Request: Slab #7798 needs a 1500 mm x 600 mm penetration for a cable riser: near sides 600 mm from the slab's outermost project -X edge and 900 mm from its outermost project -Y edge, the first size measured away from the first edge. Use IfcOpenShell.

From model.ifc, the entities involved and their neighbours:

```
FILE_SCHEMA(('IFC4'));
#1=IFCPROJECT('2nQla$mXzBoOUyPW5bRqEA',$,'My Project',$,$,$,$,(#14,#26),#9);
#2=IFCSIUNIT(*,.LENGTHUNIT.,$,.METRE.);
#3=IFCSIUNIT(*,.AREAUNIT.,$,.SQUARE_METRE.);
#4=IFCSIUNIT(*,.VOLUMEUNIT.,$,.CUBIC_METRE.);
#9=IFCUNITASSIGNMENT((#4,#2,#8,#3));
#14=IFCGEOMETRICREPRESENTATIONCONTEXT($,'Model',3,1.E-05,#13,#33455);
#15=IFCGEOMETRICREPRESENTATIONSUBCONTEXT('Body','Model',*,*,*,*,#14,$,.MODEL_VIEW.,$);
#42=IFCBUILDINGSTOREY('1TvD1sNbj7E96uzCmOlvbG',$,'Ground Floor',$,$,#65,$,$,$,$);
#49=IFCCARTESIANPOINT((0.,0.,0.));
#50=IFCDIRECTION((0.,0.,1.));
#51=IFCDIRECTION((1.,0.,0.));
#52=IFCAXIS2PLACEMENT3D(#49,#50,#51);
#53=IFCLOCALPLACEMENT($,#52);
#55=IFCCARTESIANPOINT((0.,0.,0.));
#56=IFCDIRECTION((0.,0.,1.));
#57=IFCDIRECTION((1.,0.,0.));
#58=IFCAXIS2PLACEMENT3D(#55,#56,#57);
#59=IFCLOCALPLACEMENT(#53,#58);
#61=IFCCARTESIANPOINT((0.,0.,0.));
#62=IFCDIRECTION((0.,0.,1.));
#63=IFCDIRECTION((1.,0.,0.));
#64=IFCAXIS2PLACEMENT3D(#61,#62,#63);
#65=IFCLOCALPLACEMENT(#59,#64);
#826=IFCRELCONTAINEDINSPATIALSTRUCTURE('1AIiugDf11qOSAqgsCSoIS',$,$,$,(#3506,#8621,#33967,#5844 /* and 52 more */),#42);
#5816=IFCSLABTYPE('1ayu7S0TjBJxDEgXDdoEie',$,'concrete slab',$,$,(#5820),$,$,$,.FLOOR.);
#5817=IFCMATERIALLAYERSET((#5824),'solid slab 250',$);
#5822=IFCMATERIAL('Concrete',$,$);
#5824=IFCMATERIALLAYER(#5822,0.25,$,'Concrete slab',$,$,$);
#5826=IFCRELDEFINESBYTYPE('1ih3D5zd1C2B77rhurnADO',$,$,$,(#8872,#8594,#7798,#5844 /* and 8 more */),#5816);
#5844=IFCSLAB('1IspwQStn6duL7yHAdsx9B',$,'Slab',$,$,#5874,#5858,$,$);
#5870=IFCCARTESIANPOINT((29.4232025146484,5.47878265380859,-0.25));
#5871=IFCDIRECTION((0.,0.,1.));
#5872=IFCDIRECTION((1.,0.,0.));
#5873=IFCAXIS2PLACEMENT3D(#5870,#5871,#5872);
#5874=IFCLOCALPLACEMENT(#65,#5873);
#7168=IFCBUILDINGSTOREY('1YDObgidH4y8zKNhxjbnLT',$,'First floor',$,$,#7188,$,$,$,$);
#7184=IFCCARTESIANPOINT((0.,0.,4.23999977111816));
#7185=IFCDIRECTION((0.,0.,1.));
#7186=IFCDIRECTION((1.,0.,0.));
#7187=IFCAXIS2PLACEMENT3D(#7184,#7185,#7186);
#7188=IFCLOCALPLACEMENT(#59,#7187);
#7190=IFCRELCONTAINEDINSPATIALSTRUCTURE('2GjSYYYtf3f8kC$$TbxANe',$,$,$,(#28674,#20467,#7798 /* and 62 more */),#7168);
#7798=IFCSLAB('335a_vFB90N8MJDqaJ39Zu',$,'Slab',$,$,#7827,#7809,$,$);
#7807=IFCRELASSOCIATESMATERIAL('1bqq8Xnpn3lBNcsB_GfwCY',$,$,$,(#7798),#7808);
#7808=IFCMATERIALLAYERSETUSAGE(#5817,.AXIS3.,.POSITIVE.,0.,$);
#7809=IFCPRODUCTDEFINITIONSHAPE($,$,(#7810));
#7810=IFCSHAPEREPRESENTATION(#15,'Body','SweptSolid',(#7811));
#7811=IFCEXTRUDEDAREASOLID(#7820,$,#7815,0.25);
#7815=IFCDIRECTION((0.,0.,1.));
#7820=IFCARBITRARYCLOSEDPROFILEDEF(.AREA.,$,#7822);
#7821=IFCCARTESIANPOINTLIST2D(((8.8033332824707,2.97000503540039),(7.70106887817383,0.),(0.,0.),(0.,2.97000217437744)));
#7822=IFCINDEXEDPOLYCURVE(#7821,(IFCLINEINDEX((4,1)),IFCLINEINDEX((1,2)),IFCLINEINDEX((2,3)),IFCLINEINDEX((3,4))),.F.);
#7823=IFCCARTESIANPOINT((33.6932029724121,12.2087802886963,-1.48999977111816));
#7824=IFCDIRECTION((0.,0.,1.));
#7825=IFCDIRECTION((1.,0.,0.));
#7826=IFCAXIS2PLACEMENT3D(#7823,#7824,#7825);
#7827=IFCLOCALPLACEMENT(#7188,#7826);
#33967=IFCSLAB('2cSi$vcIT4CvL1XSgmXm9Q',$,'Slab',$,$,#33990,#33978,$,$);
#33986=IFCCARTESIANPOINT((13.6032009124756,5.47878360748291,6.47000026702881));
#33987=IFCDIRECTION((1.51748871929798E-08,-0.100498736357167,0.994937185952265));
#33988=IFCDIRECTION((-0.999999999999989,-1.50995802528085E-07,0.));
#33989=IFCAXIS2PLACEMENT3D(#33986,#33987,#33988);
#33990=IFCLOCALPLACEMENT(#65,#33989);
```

```python
import numpy as np
import ifcopenshell
import ifcopenshell.api.feature
import ifcopenshell.api.geometry
import ifcopenshell.api.root
import ifcopenshell.geom
import ifcopenshell.util.placement
import ifcopenshell.util.representation
import ifcopenshell.util.shape
import ifcopenshell.util.unit

model = ifcopenshell.open("model.ifc")
unit_scale = ifcopenshell.util.unit.calculate_unit_scale(model)
settings = ifcopenshell.geom.settings()


def volume(element):
    """Net volume in cubic metres, openings subtracted."""
    shape = ifcopenshell.geom.create_shape(settings, element)
    return ifcopenshell.util.shape.get_volume(shape.geometry)


slab = model.by_guid("335a_vFB90N8MJDqaJ39Zu")
before = volume(slab)

# Extent in the slab's own axes, in metres. The edges named are its -X and -Y sides.
slab_shape = ifcopenshell.geom.create_shape(settings, slab)
vertices = ifcopenshell.util.shape.get_vertices(slab_shape.geometry)
x_min, y_min, bottom = vertices.min(axis=0)
top = vertices[:, 2].max()

opening = ifcopenshell.api.root.create_entity(model, ifc_class="IfcOpeningElement", name="Cable riser opening", predefined_type="OPENING")
context = ifcopenshell.util.representation.get_context(model, "Model", "Body", "MODEL_VIEW")
width, depth = 1.5, 0.6
outline = [(0.0, 0.0), (width, 0.0), (width, depth), (0.0, depth), (0.0, 0.0)]
# Overshoot both faces by 50 mm so the cut is clean.
shape = ifcopenshell.api.geometry.add_slab_representation(
    model, context=context, depth=top - bottom + 0.1, polyline=outline
)
ifcopenshell.api.geometry.assign_representation(model, product=opening, representation=shape)

matrix = ifcopenshell.util.placement.get_local_placement(slab.ObjectPlacement)
matrix[:, 3] = matrix @ np.append(np.array([x_min + 0.6, y_min + 0.9, bottom - 0.05]) / unit_scale, 1.0)
ifcopenshell.api.geometry.edit_object_placement(model, product=opening, matrix=matrix, is_si=False)
ifcopenshell.api.feature.add_feature(model, feature=opening, element=slab)

after = volume(slab)

print(f"slab volume {before:.3f} -> {after:.3f} m3")

model.write("model_updated.ifc")
```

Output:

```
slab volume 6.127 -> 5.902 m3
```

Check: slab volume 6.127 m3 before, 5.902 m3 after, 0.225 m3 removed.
